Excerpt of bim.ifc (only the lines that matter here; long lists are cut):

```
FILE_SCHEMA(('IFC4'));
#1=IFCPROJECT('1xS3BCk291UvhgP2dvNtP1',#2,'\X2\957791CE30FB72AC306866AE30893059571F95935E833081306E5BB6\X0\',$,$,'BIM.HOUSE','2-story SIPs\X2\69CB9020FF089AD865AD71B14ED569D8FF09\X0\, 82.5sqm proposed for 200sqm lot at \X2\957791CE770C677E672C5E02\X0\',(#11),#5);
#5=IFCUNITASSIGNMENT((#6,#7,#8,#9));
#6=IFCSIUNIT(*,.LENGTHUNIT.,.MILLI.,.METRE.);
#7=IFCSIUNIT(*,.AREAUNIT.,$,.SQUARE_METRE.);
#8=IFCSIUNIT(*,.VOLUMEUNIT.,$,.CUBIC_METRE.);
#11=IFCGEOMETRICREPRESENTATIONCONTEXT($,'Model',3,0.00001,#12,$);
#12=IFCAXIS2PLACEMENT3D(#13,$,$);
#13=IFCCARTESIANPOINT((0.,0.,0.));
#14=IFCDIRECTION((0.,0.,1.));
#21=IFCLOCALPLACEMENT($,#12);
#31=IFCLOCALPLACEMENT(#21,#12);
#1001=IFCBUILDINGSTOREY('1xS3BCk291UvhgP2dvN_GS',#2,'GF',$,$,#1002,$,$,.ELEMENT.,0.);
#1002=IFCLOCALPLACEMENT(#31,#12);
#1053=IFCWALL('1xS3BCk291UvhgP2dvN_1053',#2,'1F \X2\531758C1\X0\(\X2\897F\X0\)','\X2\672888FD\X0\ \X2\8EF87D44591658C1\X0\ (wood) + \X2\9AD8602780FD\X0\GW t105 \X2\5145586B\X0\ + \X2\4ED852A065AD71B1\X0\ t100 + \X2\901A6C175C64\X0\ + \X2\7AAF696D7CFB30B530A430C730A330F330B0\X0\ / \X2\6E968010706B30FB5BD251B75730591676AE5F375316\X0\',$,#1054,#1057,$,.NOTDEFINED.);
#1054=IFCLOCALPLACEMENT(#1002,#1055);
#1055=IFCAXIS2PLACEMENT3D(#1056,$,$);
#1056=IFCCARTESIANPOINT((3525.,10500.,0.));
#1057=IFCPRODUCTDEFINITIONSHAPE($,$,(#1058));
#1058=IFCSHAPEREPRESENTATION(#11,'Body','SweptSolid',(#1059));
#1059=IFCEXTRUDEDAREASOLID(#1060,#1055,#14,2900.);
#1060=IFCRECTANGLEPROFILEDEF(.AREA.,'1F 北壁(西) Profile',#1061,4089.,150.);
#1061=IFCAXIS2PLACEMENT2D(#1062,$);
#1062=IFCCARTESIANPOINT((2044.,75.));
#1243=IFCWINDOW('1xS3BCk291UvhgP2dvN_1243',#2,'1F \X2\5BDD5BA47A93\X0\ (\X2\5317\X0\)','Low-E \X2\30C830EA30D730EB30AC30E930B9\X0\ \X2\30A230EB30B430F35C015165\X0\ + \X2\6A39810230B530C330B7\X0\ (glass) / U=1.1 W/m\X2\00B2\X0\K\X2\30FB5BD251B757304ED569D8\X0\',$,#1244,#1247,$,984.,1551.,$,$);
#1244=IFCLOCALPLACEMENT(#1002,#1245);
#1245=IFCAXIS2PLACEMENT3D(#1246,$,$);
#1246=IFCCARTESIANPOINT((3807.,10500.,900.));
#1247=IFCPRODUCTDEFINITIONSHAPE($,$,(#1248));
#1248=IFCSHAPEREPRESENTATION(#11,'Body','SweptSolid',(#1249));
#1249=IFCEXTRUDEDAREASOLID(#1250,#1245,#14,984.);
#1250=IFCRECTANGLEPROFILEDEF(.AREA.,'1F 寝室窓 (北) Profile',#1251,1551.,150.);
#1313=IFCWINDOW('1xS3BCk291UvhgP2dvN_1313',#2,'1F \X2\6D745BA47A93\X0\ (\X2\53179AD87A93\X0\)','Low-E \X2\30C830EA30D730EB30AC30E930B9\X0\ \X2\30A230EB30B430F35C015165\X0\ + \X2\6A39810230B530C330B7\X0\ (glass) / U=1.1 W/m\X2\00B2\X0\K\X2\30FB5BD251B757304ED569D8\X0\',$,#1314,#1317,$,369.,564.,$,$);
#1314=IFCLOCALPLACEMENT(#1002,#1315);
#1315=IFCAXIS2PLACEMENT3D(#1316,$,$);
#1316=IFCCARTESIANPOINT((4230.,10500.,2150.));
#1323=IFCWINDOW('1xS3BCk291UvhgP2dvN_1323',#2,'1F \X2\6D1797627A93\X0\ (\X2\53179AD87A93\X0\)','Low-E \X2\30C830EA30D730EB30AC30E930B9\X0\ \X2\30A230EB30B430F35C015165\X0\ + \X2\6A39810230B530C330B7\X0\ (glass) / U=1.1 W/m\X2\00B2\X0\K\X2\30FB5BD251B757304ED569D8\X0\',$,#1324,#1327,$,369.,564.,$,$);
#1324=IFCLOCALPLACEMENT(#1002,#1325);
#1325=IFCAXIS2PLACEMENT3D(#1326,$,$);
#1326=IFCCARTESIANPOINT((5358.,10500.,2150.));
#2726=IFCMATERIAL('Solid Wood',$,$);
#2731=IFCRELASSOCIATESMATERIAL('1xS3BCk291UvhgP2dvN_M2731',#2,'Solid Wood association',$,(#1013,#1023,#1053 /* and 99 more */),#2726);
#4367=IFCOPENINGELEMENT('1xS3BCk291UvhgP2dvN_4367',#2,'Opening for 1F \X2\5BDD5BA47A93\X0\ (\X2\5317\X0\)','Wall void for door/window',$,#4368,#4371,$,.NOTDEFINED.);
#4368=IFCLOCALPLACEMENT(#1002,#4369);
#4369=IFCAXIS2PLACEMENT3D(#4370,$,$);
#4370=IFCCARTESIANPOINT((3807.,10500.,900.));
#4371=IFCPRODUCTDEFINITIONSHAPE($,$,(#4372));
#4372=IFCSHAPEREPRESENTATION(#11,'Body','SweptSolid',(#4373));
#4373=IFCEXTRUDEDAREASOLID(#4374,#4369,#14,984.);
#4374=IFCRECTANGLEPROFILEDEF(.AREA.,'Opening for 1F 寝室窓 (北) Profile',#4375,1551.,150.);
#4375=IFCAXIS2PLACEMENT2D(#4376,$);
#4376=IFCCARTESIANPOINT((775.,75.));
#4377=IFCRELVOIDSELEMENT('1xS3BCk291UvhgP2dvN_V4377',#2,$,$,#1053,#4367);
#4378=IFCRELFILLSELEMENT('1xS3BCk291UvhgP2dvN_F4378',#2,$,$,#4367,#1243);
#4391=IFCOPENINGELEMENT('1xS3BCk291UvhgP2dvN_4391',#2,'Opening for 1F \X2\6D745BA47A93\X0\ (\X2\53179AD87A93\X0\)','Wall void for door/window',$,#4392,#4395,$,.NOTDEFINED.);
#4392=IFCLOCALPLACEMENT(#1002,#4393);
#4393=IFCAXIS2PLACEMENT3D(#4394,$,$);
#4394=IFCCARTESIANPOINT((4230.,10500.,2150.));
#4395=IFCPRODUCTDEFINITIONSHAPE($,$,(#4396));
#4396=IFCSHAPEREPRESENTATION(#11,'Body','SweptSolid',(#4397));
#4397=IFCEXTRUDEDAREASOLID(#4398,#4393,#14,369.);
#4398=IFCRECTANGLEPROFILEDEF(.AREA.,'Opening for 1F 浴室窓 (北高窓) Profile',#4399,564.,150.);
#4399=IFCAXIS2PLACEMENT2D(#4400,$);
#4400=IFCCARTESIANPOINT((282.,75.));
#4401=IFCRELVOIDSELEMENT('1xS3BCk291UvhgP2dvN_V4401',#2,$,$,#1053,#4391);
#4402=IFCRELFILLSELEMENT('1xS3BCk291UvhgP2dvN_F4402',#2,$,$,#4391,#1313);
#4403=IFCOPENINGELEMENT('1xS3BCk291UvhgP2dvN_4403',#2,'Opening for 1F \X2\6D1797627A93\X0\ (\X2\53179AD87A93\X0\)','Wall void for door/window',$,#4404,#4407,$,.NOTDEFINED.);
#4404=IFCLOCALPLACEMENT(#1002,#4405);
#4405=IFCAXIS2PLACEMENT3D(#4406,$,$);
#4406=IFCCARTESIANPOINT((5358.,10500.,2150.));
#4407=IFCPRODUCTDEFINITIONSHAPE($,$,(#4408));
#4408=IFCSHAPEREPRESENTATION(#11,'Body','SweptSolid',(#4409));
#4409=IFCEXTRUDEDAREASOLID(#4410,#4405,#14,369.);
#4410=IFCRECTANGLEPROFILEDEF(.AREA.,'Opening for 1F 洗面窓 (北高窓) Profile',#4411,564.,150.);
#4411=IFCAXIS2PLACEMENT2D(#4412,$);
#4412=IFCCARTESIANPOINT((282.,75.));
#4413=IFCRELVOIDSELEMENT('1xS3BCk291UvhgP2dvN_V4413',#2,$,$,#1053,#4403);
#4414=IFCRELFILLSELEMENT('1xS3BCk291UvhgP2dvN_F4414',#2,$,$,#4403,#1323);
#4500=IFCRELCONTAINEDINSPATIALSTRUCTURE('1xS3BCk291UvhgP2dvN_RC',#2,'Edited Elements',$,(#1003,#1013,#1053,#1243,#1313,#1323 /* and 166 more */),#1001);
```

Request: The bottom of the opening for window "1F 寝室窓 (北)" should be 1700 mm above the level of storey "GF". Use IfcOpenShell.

```python
import numpy as np
import ifcopenshell
import ifcopenshell.api.geometry
import ifcopenshell.geom
import ifcopenshell.util.element
import ifcopenshell.util.placement
import ifcopenshell.util.shape
import ifcopenshell.util.unit

model = ifcopenshell.open("bim.ifc")
unit_scale = ifcopenshell.util.unit.calculate_unit_scale(model)

window = model.by_guid("1xS3BCk291UvhgP2dvN_1243")
opening = window.FillsVoids[0].RelatingOpeningElement
storey = ifcopenshell.util.element.get_container(window, ifc_class="IfcBuildingStorey")
level = ifcopenshell.util.placement.get_local_placement(storey.ObjectPlacement)[2, 3]

# The opening's origin need not be at the sill, so measure its lowest point.
shape = ifcopenshell.geom.create_shape(ifcopenshell.geom.settings(), opening)
bottom = ifcopenshell.util.shape.get_shape_bottom_elevation(shape, shape.geometry) / unit_scale
dz = level + 1.7 / unit_scale - bottom

shift = np.array([0.0, 0.0, dz])
# The window is not placed relative to its opening, so move both.
for product in (opening, window):
    matrix = ifcopenshell.util.placement.get_local_placement(product.ObjectPlacement)
    matrix[:3, 3] += shift
    ifcopenshell.api.geometry.edit_object_placement(model, product=product, matrix=matrix, is_si=False)

print(f"moved by {dz * unit_scale:+.3f} m")

model.write("bim_edited.ifc")
```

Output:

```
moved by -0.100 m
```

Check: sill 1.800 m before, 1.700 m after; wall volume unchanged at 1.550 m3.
